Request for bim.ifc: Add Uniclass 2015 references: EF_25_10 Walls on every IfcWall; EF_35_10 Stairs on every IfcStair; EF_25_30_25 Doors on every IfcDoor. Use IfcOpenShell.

First a look at what the model holds.

```python
import ifcopenshell

model = ifcopenshell.open("bim.ifc")
print(model.schema)
print("classifications:", [c.Name for c in model.by_type("IfcClassification")])
for ifc_class in ("IfcDoor", "IfcRoof", "IfcStair", "IfcWall", "IfcWindow"):
    print(ifc_class, len(model.by_type(ifc_class)))
```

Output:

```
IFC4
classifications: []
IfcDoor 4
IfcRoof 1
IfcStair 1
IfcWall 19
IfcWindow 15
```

```python
import ifcopenshell
import ifcopenshell.api.classification

model = ifcopenshell.open("bim.ifc")

system = ifcopenshell.api.classification.add_classification(model, classification="Uniclass 2015")

codes = {
    "IfcWall": ("EF_25_10", "Walls"),
    "IfcStair": ("EF_35_10", "Stairs"),
    "IfcDoor": ("EF_25_30_25", "Doors"),
}
for ifc_class, (code, name) in codes.items():
    products = model.by_type(ifc_class)
    ifcopenshell.api.classification.add_reference(
        model, products=products, classification=system, identification=code, name=name
    )
    print(code, len(products))

model.write("bim_updated.ifc")
```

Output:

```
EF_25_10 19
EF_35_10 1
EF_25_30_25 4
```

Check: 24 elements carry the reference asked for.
